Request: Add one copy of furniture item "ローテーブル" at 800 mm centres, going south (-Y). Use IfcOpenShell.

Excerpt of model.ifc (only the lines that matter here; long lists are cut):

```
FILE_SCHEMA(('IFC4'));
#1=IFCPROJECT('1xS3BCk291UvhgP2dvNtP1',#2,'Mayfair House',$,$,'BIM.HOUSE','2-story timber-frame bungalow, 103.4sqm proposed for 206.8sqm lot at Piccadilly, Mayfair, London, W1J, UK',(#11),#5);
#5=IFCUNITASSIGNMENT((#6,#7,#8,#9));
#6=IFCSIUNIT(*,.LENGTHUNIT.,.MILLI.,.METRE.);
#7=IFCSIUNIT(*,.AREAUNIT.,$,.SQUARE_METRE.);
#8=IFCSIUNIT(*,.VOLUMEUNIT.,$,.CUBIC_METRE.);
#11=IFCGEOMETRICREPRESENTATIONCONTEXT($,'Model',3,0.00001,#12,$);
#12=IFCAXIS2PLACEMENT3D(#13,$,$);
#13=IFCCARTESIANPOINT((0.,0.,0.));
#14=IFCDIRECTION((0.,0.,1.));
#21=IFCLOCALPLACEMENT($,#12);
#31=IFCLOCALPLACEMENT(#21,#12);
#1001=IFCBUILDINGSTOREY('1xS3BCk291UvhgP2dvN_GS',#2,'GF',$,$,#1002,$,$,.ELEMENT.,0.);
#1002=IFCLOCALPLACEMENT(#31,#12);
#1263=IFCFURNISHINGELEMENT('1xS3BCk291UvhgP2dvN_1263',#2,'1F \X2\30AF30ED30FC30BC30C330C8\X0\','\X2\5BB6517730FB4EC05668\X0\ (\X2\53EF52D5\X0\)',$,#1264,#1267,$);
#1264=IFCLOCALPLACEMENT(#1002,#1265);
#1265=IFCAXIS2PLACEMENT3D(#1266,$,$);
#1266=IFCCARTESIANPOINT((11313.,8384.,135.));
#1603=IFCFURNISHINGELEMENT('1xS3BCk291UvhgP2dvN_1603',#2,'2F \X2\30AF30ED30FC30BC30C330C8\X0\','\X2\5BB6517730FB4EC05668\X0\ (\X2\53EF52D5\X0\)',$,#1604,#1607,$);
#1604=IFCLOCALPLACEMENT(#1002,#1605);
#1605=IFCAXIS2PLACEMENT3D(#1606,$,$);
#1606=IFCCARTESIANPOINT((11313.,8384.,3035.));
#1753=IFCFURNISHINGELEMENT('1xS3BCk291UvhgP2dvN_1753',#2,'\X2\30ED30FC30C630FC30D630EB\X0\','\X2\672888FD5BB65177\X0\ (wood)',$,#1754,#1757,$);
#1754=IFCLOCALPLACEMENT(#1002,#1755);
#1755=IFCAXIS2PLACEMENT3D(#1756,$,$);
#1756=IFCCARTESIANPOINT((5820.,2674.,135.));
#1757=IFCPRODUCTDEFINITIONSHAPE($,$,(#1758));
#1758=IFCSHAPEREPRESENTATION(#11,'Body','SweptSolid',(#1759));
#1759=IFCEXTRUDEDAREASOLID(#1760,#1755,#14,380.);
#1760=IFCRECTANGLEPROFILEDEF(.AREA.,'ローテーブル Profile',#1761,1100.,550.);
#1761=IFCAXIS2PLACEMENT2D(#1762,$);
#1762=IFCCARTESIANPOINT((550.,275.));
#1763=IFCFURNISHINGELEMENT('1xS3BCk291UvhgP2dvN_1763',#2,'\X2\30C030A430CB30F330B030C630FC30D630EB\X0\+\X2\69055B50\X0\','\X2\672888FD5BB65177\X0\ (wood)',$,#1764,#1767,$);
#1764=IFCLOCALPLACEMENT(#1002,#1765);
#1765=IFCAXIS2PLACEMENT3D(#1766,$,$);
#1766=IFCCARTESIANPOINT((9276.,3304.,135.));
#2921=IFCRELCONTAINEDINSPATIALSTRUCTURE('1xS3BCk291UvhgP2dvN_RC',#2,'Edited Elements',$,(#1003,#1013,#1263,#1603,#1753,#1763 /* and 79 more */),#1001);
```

```python
import numpy as np
import ifcopenshell
import ifcopenshell.api.geometry
import ifcopenshell.api.root
import ifcopenshell.util.element
import ifcopenshell.util.placement

model = ifcopenshell.open("model.ifc")


def reuse_history(source, copy):
    """copy_class also copies each property set's owner history, people and application; keep the originals."""
    for rel in copy.IsDefinedBy:
        if rel.is_a("IfcRelDefinesByProperties") and (history := rel.RelatingPropertyDefinition.OwnerHistory):
            rel.RelatingPropertyDefinition.OwnerHistory = source.OwnerHistory
            ifcopenshell.util.element.remove_deep2(model, history)


source = model.by_guid("1xS3BCk291UvhgP2dvN_1753")
base = ifcopenshell.util.placement.get_local_placement(source.ObjectPlacement)
step = np.array([0.0, -1.0, 0.0]) * 800.0

for i in range(1, 2):
    copy = ifcopenshell.api.root.copy_class(model, product=source)
    copy.Representation = ifcopenshell.util.element.copy_deep(
        model, source.Representation, exclude=["IfcGeometricRepresentationContext", "IfcRepresentationMap"]
    )
    reuse_history(source, copy)
    matrix = base.copy()
    matrix[:3, 3] += i * step
    print("added at", matrix[:3, 3].round(3) + 0.0)
    ifcopenshell.api.geometry.edit_object_placement(model, product=copy, matrix=matrix, is_si=False)

model.write("model_updated.ifc")
```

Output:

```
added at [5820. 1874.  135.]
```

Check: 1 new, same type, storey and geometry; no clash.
